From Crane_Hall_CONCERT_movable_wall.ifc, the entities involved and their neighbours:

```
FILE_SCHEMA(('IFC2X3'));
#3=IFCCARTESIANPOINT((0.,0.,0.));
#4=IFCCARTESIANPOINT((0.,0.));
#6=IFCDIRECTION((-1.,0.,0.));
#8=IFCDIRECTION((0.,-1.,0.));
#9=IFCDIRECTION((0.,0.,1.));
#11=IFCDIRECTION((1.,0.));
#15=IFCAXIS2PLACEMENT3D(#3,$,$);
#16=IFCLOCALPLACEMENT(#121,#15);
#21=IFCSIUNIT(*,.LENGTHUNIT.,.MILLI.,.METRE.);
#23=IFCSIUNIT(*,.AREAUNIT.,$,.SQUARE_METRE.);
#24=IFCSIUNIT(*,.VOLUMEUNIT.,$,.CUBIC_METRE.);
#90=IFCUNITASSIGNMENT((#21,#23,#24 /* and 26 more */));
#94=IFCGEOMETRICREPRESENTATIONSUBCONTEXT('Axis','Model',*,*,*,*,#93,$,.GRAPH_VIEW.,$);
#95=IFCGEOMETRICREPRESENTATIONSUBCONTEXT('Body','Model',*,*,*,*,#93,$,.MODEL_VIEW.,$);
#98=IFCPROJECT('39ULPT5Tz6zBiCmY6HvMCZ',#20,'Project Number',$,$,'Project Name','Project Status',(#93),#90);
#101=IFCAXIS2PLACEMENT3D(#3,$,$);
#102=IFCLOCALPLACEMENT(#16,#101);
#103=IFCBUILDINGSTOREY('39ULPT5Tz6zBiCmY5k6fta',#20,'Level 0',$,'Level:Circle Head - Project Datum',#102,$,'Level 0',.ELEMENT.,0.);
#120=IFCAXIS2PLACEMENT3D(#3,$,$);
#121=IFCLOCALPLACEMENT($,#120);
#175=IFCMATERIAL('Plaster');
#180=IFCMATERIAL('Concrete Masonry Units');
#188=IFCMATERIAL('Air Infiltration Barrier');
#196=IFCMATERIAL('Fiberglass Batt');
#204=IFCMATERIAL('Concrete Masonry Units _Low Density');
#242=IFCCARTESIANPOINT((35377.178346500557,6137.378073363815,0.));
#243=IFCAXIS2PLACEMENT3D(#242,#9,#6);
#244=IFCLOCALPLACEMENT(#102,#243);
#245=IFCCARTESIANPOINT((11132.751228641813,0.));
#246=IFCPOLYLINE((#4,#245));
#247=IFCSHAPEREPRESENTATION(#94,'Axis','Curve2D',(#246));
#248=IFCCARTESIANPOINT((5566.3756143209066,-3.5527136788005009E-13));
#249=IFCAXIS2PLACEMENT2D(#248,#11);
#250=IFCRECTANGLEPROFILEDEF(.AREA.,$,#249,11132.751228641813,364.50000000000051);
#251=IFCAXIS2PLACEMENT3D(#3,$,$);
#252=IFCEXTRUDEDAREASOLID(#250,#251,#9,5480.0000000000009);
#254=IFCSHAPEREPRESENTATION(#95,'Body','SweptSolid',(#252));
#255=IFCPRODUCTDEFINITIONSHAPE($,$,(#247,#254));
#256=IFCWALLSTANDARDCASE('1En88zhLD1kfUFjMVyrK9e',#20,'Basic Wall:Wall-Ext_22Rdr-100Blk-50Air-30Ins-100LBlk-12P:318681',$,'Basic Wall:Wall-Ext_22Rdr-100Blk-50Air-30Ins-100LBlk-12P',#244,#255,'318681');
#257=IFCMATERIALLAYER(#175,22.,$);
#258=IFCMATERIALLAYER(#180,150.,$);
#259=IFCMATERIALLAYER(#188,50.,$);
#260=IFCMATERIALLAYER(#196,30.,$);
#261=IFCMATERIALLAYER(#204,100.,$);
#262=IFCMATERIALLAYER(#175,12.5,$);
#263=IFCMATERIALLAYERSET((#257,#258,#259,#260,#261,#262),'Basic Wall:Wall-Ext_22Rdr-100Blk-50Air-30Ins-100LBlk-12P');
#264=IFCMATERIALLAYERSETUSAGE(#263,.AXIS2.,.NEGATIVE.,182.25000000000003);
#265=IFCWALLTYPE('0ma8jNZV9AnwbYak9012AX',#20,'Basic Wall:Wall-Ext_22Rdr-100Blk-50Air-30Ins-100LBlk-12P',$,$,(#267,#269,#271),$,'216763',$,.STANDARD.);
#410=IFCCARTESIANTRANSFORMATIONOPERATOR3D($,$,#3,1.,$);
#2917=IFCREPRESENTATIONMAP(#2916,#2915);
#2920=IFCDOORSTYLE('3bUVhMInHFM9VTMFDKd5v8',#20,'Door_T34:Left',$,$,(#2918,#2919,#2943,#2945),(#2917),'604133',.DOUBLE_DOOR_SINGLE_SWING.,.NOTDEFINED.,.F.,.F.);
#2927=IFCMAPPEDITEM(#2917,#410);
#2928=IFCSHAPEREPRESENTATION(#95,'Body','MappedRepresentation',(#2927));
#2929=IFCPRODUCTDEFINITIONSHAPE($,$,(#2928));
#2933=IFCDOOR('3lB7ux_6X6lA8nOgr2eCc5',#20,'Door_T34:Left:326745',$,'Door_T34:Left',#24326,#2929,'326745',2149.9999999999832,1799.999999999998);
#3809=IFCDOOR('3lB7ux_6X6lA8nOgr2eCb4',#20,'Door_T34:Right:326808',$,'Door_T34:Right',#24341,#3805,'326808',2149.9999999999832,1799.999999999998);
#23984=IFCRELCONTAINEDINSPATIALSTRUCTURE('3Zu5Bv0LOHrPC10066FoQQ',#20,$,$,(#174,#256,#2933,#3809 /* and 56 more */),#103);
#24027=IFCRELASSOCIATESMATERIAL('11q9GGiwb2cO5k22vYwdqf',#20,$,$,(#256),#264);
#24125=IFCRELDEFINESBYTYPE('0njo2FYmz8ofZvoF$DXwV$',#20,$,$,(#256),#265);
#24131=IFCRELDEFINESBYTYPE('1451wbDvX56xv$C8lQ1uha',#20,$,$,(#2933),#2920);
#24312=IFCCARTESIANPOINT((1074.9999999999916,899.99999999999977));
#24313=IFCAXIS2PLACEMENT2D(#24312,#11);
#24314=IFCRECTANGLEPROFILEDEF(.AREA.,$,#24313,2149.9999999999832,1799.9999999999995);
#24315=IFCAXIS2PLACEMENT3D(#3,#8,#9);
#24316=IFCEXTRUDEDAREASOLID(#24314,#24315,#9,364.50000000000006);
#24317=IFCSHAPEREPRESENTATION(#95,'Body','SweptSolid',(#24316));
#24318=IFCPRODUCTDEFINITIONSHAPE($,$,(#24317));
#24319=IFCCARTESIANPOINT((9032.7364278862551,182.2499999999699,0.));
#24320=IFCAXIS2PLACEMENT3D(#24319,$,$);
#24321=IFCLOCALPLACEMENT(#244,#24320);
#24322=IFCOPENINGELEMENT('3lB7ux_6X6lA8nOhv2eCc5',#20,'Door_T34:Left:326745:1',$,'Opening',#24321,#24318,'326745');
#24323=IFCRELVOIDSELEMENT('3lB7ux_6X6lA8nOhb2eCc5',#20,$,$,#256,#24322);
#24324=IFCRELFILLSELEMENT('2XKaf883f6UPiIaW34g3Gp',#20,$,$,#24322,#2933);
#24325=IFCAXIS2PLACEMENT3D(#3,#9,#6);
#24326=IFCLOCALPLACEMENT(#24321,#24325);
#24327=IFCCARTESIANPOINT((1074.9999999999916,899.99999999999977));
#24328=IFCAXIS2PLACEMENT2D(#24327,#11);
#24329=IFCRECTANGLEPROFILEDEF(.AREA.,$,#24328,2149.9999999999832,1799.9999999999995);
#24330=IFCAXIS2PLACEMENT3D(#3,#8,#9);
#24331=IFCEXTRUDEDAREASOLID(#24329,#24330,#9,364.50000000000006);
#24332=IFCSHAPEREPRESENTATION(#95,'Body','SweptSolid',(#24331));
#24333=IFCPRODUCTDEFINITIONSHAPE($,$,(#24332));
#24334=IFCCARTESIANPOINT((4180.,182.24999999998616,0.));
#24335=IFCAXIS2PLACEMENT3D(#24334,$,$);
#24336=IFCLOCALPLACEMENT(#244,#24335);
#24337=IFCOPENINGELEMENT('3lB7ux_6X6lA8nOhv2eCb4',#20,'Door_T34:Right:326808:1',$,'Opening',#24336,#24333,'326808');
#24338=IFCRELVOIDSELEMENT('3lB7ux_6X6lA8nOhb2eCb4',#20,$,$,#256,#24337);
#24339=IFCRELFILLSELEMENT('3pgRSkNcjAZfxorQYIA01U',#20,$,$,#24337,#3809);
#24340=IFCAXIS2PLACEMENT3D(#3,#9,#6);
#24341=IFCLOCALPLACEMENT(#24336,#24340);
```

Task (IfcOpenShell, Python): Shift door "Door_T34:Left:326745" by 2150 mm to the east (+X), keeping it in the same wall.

```python
import ifcopenshell
import ifcopenshell.api.geometry
import ifcopenshell.util.placement
import ifcopenshell.util.unit

model = ifcopenshell.open("Crane_Hall_CONCERT_movable_wall.ifc")
unit_scale = ifcopenshell.util.unit.calculate_unit_scale(model)

door = model.by_guid("3lB7ux_6X6lA8nOgr2eCc5")
opening = door.FillsVoids[0].RelatingOpeningElement
wall = opening.VoidsElements[0].RelatingBuildingElement

wall_matrix = ifcopenshell.util.placement.get_local_placement(wall.ObjectPlacement)
shift = wall_matrix[:3, 0] * -2.15 / unit_scale
before = ifcopenshell.util.placement.get_local_placement(door.ObjectPlacement)[:3, 3].copy()

# The door is placed relative to its opening, so it follows when the opening moves.
matrix = ifcopenshell.util.placement.get_local_placement(opening.ObjectPlacement)
matrix[:3, 3] += shift
ifcopenshell.api.geometry.edit_object_placement(
    model, product=opening, matrix=matrix, is_si=False, should_transform_children=True
)

after = ifcopenshell.util.placement.get_local_placement(door.ObjectPlacement)[:3, 3]
print("door moved by", (after - before).round(3) + 0.0)

model.write("Crane_Hall_CONCERT_movable_wall_updated.ifc")
```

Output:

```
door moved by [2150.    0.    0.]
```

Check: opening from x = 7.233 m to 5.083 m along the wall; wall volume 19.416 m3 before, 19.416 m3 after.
